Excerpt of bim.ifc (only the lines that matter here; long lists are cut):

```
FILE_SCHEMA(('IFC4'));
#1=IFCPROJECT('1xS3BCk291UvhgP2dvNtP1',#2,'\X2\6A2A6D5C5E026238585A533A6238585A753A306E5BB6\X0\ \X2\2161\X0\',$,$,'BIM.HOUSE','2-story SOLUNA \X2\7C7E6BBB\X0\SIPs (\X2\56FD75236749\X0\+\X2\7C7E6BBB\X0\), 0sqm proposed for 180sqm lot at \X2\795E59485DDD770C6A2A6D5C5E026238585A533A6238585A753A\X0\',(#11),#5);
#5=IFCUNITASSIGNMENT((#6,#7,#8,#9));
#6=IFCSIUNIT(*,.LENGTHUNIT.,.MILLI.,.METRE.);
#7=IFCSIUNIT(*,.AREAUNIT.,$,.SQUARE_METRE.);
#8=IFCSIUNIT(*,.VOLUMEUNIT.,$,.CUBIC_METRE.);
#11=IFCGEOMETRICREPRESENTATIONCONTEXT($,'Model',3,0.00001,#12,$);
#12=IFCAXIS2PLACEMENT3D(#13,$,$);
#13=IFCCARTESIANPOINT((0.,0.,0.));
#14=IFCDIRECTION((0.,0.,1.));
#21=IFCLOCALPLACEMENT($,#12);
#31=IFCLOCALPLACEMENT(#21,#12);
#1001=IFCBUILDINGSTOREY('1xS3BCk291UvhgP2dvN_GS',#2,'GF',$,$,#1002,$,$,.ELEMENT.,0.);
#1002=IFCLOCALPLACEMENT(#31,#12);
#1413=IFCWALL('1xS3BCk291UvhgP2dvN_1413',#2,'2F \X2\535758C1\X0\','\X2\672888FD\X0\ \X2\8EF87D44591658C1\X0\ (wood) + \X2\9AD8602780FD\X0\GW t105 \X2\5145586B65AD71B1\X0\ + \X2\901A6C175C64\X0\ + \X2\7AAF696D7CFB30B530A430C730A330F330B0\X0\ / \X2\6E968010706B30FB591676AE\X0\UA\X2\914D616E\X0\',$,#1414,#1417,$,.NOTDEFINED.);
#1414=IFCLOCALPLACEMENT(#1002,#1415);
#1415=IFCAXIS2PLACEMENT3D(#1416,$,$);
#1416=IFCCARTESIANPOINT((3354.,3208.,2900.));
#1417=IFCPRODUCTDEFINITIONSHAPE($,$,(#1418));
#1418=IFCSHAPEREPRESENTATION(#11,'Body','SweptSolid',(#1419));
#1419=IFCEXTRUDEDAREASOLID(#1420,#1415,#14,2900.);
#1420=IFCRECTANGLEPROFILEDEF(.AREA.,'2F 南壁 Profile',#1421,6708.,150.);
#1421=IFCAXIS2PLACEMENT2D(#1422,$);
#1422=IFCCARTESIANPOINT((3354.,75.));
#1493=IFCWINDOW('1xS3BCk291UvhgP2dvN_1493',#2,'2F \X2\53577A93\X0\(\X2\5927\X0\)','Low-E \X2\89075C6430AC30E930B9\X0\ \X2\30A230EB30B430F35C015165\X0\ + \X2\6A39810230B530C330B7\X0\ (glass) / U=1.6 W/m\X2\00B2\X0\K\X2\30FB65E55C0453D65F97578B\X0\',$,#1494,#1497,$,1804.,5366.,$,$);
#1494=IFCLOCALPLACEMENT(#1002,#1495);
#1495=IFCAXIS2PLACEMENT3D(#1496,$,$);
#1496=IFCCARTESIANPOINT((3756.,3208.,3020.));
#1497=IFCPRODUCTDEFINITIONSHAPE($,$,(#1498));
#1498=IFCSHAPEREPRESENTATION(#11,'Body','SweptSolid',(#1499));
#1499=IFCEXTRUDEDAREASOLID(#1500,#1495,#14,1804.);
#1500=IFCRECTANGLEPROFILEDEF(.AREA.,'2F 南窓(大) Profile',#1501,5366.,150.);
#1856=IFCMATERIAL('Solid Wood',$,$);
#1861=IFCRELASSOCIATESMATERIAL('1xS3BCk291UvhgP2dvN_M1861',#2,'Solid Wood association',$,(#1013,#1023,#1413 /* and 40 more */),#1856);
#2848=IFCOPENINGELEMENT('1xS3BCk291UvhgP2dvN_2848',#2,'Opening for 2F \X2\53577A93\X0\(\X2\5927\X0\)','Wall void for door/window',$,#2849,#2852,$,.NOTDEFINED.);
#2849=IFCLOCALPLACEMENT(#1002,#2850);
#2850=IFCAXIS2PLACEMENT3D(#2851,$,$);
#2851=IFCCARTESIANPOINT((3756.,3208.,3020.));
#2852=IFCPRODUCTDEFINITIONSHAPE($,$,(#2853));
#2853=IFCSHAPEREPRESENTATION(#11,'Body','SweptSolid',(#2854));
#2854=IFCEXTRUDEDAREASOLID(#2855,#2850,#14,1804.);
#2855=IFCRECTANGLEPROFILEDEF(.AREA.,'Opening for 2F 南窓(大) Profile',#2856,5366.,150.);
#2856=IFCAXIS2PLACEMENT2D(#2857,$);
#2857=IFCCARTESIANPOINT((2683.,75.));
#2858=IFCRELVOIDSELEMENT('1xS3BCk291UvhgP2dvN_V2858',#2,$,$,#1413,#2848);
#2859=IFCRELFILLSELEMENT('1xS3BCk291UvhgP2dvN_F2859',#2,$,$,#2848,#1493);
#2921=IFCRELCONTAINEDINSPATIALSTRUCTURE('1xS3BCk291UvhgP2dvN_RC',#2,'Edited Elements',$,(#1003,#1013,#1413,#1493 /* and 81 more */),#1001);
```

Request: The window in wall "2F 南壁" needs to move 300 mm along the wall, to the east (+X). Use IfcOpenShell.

```python
import ifcopenshell
import ifcopenshell.api.geometry
import ifcopenshell.util.placement

model = ifcopenshell.open("bim.ifc")

window = model.by_guid("1xS3BCk291UvhgP2dvN_1493")
opening = window.FillsVoids[0].RelatingOpeningElement
wall = opening.VoidsElements[0].RelatingBuildingElement

wall_matrix = ifcopenshell.util.placement.get_local_placement(wall.ObjectPlacement)
shift = wall_matrix[:3, 0] * 300.0
before = ifcopenshell.util.placement.get_local_placement(window.ObjectPlacement)[:3, 3].copy()

# The window is not placed relative to its opening, so move both.
for product in (opening, window):
    matrix = ifcopenshell.util.placement.get_local_placement(product.ObjectPlacement)
    matrix[:3, 3] += shift
    ifcopenshell.api.geometry.edit_object_placement(model, product=product, matrix=matrix, is_si=False)

after = ifcopenshell.util.placement.get_local_placement(window.ObjectPlacement)[:3, 3]
print("window moved by", (after - before).round(3) + 0.0)

model.write("bim_v2.ifc")
```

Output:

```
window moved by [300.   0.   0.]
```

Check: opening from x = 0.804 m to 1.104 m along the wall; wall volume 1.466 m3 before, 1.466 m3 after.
